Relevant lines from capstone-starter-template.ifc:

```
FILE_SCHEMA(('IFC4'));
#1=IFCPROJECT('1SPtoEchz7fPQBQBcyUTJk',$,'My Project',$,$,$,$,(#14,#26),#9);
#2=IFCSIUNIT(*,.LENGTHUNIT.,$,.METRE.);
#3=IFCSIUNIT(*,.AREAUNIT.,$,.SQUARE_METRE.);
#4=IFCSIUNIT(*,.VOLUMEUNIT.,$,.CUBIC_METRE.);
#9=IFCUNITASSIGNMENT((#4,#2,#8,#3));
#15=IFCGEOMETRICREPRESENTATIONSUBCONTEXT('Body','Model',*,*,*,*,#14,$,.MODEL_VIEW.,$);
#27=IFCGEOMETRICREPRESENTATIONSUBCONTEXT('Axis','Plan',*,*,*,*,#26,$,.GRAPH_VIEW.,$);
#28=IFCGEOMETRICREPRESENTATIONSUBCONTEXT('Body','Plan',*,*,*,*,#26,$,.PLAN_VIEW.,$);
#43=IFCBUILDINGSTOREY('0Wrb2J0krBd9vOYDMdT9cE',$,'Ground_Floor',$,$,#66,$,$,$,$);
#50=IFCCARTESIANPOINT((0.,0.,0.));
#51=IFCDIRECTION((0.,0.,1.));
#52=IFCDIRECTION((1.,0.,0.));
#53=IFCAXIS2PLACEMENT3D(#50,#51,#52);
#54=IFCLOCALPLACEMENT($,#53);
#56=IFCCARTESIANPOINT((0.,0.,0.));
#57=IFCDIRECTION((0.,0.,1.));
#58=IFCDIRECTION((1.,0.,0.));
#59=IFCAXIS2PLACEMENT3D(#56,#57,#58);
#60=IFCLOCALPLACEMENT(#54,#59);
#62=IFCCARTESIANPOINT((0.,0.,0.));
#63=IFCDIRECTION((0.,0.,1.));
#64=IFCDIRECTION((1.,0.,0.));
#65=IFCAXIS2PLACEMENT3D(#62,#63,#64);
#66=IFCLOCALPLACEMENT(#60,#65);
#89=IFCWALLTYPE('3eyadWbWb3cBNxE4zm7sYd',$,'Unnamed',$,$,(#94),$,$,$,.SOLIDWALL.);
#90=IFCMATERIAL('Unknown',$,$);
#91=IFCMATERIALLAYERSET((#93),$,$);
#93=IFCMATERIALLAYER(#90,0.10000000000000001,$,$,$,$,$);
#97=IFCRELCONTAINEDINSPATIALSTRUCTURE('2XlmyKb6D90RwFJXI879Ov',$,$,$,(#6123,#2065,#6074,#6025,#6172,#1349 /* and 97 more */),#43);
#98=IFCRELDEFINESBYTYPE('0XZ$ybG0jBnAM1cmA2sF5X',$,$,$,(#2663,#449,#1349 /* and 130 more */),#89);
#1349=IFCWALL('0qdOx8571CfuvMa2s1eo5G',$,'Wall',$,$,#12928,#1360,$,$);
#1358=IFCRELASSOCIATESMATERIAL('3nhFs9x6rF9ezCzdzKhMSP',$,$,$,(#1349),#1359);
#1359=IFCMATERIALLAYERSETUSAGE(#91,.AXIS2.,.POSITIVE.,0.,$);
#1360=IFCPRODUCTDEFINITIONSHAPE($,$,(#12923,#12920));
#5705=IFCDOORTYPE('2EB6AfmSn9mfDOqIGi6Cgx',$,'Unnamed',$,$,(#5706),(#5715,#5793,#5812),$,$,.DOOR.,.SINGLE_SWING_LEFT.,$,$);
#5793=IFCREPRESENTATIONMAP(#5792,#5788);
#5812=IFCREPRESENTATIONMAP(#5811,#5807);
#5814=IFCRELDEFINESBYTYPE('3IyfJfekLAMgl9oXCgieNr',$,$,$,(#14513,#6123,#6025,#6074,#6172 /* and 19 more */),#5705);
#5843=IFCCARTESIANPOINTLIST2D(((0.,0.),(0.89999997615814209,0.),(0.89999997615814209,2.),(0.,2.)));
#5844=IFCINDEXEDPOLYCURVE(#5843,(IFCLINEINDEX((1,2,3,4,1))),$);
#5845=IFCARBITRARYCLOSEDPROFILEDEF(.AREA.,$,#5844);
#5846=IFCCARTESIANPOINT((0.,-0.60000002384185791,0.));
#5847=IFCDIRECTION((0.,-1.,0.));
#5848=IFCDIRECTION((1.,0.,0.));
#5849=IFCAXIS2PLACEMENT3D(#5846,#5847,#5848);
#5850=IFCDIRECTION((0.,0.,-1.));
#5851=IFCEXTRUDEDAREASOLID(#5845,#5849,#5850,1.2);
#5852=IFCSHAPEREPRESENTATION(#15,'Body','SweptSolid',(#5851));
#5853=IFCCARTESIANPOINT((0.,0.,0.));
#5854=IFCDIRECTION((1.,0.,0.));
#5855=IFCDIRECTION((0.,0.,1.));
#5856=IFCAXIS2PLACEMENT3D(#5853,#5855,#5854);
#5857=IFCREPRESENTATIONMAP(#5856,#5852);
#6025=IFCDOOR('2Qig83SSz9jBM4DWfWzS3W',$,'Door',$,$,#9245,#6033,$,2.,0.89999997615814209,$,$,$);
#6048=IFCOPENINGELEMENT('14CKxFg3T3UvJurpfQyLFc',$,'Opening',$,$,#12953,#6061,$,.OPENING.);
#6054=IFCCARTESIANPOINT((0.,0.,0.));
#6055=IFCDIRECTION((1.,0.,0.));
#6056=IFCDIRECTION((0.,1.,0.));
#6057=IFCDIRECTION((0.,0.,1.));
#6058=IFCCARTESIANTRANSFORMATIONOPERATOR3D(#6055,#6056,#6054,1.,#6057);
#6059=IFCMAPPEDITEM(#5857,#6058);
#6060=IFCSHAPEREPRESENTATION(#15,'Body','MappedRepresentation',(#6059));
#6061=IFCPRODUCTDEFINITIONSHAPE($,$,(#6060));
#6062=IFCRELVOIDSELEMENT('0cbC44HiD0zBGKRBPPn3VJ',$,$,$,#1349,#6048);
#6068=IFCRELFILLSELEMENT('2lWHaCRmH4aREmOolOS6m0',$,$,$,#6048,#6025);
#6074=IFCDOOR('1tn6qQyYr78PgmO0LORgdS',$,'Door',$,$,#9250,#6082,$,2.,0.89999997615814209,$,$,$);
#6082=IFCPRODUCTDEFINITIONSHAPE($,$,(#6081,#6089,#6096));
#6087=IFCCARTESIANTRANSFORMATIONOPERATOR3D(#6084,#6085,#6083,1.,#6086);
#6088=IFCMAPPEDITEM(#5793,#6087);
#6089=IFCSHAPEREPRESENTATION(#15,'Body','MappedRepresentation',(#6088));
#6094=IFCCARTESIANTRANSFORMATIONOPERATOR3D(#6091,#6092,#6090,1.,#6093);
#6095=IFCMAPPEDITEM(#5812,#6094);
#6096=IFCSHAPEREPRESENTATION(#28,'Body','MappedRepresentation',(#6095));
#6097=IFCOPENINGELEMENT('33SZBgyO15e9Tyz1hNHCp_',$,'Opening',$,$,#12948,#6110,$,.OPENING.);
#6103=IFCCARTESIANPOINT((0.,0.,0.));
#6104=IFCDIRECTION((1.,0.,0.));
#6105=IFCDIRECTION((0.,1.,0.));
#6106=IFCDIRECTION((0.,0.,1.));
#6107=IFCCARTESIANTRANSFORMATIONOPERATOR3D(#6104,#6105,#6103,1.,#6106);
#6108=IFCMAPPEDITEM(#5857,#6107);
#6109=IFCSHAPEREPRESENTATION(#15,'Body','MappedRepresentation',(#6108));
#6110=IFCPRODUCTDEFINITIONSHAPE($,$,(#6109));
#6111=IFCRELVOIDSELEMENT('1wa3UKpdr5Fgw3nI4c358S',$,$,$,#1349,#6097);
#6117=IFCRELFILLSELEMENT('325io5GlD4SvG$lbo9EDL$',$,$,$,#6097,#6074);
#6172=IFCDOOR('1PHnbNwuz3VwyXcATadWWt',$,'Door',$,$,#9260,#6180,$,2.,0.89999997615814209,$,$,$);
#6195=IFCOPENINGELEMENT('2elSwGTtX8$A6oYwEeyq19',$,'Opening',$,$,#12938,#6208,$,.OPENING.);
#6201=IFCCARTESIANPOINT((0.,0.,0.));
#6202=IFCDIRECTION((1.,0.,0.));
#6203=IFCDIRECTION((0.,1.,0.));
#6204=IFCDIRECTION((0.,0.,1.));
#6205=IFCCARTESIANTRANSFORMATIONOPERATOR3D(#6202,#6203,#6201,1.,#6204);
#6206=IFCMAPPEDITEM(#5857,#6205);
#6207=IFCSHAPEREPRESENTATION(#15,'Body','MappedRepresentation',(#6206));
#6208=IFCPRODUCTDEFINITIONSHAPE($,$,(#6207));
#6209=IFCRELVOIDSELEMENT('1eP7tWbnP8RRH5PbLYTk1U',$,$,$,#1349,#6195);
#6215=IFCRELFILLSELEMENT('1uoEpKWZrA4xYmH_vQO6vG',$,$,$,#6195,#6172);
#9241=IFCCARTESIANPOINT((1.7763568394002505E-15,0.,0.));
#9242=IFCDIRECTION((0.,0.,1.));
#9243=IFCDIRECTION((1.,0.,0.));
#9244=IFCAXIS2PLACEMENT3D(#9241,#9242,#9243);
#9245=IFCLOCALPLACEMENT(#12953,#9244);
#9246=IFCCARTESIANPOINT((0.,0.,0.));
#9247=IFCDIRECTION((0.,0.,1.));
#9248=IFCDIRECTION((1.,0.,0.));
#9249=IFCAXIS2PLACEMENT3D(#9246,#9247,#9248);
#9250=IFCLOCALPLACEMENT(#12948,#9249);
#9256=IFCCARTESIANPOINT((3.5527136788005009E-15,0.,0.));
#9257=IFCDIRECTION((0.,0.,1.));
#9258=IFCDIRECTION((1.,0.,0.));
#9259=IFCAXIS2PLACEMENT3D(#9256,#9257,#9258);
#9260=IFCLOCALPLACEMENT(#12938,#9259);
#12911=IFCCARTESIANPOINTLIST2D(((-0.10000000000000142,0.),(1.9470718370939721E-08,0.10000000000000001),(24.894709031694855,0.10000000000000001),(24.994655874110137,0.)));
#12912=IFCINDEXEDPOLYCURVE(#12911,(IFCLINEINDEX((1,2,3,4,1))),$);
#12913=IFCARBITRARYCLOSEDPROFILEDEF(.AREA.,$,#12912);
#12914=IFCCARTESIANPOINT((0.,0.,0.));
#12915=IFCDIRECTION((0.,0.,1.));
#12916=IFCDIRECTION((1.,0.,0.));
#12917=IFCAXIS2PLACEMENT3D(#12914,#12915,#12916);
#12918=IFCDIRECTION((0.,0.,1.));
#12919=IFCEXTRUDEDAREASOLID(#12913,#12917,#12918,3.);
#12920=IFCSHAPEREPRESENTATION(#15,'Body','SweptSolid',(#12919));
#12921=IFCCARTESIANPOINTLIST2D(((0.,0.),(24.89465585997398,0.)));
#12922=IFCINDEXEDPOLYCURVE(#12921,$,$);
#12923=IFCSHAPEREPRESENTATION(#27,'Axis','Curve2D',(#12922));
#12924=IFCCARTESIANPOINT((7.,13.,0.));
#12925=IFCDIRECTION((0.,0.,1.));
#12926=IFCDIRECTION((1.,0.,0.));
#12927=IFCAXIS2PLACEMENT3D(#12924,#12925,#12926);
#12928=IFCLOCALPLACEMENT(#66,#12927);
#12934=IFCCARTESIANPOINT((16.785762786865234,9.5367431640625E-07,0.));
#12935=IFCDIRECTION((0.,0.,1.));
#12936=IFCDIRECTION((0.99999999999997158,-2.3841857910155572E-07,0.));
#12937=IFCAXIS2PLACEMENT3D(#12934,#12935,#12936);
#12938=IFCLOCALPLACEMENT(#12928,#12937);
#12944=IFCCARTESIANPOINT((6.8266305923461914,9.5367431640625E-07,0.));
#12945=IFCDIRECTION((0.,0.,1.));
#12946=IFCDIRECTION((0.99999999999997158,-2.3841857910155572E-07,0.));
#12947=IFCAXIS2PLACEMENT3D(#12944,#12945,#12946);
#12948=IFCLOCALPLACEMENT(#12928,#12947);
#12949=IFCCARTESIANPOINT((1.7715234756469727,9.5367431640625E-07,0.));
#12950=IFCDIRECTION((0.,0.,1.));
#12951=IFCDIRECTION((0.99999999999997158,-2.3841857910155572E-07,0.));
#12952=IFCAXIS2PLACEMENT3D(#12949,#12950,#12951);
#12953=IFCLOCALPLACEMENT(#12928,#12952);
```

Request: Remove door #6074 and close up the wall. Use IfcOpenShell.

```python
import ifcopenshell
import ifcopenshell.api.feature
import ifcopenshell.api.root
import ifcopenshell.geom
import ifcopenshell.util.shape

model = ifcopenshell.open("capstone-starter-template.ifc")
settings = ifcopenshell.geom.settings()


def volume(element):
    """Net volume in cubic metres, openings subtracted."""
    shape = ifcopenshell.geom.create_shape(settings, element)
    return ifcopenshell.util.shape.get_volume(shape.geometry)


door = model.by_guid("1tn6qQyYr78PgmO0LORgdS")
opening = door.FillsVoids[0].RelatingOpeningElement
wall = opening.VoidsElements[0].RelatingBuildingElement
before = volume(wall)

ifcopenshell.api.root.remove_product(model, product=door)
ifcopenshell.api.feature.remove_feature(model, feature=opening)

after = volume(wall)

print(f"wall volume {before:.3f} -> {after:.3f} m3")

model.write("capstone-starter-template-out.ifc")
```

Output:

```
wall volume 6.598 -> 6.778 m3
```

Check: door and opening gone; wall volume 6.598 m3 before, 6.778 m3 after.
